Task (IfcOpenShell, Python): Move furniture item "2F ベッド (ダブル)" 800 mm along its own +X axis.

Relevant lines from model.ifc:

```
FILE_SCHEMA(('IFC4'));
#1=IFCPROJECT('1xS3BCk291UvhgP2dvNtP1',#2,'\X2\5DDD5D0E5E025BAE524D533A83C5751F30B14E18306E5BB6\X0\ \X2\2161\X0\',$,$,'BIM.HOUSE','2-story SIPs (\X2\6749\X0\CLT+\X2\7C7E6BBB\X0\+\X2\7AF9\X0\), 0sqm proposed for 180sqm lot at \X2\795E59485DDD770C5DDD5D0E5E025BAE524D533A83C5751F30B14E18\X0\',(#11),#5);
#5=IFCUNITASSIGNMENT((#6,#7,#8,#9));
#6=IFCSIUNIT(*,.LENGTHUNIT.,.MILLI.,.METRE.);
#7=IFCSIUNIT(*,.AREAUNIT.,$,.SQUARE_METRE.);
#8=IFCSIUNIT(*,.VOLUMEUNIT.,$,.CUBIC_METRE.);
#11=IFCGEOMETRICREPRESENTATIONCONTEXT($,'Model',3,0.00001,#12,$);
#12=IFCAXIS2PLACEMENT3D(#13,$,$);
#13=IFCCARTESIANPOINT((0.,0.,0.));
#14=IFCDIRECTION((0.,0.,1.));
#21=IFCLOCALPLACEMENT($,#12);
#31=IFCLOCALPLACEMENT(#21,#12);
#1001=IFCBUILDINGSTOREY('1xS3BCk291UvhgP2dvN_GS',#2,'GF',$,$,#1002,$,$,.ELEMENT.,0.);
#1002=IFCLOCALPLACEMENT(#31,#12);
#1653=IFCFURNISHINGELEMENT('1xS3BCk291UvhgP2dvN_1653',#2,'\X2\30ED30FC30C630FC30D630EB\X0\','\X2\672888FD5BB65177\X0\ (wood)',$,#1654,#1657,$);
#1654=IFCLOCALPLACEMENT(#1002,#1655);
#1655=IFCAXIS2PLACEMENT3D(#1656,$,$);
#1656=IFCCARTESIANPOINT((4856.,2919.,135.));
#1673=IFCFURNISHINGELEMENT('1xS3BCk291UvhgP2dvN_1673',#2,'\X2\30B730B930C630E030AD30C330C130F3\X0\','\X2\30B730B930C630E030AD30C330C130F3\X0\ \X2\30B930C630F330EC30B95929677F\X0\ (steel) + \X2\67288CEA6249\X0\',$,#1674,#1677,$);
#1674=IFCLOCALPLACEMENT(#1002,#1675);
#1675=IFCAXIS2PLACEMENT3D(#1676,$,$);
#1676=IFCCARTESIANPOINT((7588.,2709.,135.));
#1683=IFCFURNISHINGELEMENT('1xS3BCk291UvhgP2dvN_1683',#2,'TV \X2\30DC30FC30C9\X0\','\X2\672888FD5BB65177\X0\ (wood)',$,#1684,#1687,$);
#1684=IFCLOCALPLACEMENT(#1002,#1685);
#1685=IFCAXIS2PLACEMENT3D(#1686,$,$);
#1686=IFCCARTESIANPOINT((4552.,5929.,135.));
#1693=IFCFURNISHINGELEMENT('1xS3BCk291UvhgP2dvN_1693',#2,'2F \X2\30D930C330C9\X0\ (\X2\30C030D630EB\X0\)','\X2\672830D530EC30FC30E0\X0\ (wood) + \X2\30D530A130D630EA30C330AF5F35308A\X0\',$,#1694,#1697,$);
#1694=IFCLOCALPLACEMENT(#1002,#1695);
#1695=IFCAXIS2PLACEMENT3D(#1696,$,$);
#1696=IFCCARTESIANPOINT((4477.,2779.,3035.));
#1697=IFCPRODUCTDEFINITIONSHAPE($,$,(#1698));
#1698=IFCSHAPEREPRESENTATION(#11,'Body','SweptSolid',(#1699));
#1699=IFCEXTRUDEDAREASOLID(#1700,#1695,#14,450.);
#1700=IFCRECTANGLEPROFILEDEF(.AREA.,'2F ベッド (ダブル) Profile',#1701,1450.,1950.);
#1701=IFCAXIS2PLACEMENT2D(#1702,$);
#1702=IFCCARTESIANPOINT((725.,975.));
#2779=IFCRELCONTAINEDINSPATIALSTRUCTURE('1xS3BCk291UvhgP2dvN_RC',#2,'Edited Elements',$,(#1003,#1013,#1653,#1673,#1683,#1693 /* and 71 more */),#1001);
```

```python
import ifcopenshell
import ifcopenshell.api.geometry
import ifcopenshell.util.placement

model = ifcopenshell.open("model.ifc")

item = model.by_guid("1xS3BCk291UvhgP2dvN_1693")
matrix = ifcopenshell.util.placement.get_local_placement(item.ObjectPlacement)
matrix[:3, 3] += matrix[:3, 0] * 800.0
ifcopenshell.api.geometry.edit_object_placement(model, product=item, matrix=matrix, is_si=False)

print(ifcopenshell.util.placement.get_local_placement(item.ObjectPlacement).round(3) + 0.0)

model.write("model_v2.ifc")
```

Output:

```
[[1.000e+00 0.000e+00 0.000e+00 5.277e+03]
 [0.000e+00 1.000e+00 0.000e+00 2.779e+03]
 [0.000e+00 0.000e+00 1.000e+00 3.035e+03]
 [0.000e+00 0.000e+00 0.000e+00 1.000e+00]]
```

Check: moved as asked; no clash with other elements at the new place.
